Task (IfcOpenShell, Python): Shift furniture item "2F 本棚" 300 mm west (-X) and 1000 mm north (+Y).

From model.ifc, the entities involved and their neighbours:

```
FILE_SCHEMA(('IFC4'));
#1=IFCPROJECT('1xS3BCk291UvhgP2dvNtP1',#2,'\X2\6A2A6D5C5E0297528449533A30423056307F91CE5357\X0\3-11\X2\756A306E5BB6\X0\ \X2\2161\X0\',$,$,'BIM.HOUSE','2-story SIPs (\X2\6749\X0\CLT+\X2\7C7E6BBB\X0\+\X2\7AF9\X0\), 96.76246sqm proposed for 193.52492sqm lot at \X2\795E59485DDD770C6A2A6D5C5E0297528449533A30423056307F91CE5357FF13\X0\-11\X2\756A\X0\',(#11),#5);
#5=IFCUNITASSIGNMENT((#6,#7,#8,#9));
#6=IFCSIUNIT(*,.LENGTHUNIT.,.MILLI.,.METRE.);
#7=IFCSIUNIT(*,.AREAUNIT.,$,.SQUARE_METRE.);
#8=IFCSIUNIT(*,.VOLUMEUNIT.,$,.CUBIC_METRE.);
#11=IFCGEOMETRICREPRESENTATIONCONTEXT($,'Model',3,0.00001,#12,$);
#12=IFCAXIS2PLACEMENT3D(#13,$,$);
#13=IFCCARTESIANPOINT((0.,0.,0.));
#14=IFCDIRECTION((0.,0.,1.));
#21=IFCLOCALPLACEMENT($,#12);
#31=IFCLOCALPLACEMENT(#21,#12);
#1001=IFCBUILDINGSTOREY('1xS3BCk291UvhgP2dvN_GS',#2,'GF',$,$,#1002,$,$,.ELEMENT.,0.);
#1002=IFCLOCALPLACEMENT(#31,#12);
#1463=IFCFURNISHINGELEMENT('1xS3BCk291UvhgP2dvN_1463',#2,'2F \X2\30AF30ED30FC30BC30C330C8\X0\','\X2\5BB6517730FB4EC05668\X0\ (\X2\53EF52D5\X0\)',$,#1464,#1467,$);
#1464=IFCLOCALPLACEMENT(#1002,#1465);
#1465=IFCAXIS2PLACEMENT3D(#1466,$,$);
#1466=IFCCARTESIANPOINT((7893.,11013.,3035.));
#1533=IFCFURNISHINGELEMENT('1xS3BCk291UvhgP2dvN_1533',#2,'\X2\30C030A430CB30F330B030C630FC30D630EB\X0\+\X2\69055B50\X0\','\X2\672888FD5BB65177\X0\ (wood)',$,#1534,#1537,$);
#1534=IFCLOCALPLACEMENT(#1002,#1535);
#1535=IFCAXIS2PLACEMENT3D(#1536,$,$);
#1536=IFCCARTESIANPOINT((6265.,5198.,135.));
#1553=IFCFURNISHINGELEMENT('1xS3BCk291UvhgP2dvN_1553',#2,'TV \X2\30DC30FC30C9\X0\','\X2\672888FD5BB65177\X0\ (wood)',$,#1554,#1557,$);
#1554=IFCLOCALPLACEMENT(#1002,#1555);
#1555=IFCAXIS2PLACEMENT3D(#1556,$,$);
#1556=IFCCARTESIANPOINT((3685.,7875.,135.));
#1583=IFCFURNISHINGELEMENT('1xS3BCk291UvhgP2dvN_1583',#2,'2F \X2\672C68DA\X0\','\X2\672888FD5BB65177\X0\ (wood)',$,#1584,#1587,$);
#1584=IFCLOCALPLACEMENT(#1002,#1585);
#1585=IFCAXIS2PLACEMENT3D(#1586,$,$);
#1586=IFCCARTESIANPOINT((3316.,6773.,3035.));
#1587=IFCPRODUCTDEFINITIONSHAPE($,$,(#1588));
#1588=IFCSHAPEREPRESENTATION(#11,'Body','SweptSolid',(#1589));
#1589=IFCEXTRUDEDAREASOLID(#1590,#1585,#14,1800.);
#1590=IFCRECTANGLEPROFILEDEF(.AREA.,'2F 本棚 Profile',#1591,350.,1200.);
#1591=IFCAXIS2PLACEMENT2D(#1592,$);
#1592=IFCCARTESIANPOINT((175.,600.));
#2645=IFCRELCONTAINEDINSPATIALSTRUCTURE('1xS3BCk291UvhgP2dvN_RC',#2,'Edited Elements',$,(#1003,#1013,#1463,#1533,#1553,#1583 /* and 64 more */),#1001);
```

```python
import ifcopenshell
import ifcopenshell.api.geometry
import ifcopenshell.util.placement
import ifcopenshell.util.unit

model = ifcopenshell.open("model.ifc")
unit_scale = ifcopenshell.util.unit.calculate_unit_scale(model)

item = model.by_guid("1xS3BCk291UvhgP2dvN_1583")
matrix = ifcopenshell.util.placement.get_local_placement(item.ObjectPlacement)
matrix[0, 3] -= 0.3 / unit_scale
matrix[1, 3] += 1 / unit_scale
ifcopenshell.api.geometry.edit_object_placement(model, product=item, matrix=matrix, is_si=False)

print(ifcopenshell.util.placement.get_local_placement(item.ObjectPlacement).round(3) + 0.0)

model.write("model-out.ifc")
```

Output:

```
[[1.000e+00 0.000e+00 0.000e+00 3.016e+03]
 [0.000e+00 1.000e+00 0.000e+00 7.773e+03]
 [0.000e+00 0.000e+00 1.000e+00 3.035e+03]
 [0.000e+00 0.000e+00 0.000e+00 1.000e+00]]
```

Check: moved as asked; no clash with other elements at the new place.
